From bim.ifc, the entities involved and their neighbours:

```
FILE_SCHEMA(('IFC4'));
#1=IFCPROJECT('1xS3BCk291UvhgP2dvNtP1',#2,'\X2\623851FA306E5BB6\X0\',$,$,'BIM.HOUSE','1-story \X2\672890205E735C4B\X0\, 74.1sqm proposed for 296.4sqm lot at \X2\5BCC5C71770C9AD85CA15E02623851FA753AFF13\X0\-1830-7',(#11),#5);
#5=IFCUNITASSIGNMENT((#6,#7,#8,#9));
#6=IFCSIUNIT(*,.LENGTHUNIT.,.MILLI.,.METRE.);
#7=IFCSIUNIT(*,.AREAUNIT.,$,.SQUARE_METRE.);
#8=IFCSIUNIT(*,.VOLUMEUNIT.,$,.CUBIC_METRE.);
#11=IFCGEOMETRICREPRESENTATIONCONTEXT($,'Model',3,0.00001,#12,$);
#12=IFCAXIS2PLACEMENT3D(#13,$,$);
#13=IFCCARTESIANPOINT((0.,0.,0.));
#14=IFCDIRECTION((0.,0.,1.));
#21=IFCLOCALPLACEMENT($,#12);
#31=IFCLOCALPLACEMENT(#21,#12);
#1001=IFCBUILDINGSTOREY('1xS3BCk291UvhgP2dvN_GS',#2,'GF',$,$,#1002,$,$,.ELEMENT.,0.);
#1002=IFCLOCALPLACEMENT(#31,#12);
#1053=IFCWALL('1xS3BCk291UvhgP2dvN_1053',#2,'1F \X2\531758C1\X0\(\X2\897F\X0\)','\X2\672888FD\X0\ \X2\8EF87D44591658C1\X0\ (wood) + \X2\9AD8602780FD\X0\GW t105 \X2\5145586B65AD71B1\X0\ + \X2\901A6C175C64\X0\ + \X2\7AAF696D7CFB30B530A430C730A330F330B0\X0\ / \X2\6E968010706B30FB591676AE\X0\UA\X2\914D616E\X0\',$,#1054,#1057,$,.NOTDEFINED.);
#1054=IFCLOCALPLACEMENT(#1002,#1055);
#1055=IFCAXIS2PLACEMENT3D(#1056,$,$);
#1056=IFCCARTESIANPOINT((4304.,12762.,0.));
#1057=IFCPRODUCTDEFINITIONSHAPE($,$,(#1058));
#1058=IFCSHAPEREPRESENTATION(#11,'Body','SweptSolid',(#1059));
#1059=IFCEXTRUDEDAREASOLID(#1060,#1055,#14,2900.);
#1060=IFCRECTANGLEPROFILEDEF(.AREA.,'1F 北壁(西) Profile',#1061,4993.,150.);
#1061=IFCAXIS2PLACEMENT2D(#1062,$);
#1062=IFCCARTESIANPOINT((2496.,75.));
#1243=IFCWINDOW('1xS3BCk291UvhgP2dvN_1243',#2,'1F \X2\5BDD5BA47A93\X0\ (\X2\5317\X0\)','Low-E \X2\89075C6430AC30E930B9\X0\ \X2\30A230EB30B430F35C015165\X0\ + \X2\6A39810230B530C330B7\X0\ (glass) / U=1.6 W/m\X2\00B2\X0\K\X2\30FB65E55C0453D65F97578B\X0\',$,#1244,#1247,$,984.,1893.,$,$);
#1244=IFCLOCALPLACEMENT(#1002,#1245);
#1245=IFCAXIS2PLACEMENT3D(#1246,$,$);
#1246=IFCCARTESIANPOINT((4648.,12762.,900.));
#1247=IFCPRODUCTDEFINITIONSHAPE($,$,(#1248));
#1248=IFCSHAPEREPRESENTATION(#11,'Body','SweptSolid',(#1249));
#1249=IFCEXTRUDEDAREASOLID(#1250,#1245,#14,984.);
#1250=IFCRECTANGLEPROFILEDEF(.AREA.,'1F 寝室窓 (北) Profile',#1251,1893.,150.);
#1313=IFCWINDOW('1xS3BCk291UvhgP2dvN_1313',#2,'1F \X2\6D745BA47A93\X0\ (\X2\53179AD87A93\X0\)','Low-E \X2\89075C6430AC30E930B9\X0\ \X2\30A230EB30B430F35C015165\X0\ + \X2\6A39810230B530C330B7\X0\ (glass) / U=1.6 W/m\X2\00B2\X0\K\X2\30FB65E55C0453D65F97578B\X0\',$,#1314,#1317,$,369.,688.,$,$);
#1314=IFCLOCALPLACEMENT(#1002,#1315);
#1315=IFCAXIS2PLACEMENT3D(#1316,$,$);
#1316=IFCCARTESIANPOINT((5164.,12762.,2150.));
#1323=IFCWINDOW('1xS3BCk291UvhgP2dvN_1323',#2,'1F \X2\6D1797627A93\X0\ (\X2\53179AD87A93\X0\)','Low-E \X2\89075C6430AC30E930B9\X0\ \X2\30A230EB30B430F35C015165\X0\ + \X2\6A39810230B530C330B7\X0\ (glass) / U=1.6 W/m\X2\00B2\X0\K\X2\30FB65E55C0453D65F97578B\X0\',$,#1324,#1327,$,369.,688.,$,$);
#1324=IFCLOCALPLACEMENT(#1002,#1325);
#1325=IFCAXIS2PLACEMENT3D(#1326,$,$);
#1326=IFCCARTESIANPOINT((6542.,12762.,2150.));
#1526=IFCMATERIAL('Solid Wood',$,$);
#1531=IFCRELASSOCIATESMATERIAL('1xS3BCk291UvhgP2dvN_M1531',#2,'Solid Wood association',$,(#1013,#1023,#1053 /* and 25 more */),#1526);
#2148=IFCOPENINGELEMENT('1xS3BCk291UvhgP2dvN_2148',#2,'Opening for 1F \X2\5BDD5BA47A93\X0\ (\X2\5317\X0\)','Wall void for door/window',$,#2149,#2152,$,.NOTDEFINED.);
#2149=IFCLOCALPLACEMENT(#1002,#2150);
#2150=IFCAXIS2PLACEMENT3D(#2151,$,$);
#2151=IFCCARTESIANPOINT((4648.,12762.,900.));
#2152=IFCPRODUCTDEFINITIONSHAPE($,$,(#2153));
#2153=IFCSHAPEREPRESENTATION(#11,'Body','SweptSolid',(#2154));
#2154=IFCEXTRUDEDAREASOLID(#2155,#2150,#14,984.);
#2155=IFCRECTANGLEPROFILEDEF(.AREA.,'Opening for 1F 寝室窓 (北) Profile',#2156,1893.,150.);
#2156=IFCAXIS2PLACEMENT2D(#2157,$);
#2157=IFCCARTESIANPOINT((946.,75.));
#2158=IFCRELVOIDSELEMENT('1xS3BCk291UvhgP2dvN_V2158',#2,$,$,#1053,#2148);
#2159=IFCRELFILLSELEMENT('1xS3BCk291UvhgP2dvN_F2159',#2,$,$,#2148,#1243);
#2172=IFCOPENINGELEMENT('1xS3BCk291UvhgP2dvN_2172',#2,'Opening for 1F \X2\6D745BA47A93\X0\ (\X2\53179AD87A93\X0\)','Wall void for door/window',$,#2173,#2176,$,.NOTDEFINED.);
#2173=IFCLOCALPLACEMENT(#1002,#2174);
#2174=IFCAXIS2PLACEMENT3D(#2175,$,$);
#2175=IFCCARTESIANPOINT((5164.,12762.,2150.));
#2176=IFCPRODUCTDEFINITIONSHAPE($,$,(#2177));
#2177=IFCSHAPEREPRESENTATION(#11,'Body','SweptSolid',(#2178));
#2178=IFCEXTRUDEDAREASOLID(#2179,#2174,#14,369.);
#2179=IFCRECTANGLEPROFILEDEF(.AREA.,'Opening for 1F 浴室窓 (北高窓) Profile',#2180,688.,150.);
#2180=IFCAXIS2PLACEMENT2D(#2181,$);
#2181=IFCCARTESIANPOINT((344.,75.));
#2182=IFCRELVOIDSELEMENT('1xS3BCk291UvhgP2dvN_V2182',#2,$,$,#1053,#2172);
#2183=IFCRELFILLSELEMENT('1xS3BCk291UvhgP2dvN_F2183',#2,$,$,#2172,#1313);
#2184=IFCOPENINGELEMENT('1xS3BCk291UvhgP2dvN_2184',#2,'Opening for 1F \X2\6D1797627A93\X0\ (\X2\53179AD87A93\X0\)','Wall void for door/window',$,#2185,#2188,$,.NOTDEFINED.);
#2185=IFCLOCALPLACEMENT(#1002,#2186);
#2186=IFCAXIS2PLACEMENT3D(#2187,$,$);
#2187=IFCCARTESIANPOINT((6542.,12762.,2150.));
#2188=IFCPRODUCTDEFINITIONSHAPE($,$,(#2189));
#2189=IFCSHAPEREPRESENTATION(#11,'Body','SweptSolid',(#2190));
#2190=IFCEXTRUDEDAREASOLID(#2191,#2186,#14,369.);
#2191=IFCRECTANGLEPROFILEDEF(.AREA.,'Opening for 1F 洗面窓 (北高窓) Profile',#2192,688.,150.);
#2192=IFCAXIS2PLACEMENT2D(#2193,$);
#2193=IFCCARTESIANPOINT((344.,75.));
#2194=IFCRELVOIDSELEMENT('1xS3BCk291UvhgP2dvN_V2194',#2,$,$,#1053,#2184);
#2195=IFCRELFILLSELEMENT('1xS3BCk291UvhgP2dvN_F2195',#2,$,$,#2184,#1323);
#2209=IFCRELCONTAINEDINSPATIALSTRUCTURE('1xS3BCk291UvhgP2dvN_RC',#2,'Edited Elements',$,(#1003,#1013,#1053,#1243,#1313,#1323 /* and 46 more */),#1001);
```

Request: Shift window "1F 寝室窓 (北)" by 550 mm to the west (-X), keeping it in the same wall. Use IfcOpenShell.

```python
import ifcopenshell
import ifcopenshell.api.geometry
import ifcopenshell.util.placement
import ifcopenshell.util.unit

model = ifcopenshell.open("bim.ifc")
unit_scale = ifcopenshell.util.unit.calculate_unit_scale(model)

window = model.by_guid("1xS3BCk291UvhgP2dvN_1243")
opening = window.FillsVoids[0].RelatingOpeningElement
wall = opening.VoidsElements[0].RelatingBuildingElement

wall_matrix = ifcopenshell.util.placement.get_local_placement(wall.ObjectPlacement)
shift = wall_matrix[:3, 0] * -0.55 / unit_scale
before = ifcopenshell.util.placement.get_local_placement(window.ObjectPlacement)[:3, 3].copy()

# The window is not placed relative to its opening, so move both.
for product in (opening, window):
    matrix = ifcopenshell.util.placement.get_local_placement(product.ObjectPlacement)
    matrix[:3, 3] += shift
    ifcopenshell.api.geometry.edit_object_placement(model, product=product, matrix=matrix, is_si=False)

after = ifcopenshell.util.placement.get_local_placement(window.ObjectPlacement)[:3, 3]
print("window moved by", (after - before).round(3) + 0.0)

model.write("bim_v2.ifc")
```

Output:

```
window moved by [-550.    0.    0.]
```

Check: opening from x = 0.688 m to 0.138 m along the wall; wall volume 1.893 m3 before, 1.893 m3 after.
